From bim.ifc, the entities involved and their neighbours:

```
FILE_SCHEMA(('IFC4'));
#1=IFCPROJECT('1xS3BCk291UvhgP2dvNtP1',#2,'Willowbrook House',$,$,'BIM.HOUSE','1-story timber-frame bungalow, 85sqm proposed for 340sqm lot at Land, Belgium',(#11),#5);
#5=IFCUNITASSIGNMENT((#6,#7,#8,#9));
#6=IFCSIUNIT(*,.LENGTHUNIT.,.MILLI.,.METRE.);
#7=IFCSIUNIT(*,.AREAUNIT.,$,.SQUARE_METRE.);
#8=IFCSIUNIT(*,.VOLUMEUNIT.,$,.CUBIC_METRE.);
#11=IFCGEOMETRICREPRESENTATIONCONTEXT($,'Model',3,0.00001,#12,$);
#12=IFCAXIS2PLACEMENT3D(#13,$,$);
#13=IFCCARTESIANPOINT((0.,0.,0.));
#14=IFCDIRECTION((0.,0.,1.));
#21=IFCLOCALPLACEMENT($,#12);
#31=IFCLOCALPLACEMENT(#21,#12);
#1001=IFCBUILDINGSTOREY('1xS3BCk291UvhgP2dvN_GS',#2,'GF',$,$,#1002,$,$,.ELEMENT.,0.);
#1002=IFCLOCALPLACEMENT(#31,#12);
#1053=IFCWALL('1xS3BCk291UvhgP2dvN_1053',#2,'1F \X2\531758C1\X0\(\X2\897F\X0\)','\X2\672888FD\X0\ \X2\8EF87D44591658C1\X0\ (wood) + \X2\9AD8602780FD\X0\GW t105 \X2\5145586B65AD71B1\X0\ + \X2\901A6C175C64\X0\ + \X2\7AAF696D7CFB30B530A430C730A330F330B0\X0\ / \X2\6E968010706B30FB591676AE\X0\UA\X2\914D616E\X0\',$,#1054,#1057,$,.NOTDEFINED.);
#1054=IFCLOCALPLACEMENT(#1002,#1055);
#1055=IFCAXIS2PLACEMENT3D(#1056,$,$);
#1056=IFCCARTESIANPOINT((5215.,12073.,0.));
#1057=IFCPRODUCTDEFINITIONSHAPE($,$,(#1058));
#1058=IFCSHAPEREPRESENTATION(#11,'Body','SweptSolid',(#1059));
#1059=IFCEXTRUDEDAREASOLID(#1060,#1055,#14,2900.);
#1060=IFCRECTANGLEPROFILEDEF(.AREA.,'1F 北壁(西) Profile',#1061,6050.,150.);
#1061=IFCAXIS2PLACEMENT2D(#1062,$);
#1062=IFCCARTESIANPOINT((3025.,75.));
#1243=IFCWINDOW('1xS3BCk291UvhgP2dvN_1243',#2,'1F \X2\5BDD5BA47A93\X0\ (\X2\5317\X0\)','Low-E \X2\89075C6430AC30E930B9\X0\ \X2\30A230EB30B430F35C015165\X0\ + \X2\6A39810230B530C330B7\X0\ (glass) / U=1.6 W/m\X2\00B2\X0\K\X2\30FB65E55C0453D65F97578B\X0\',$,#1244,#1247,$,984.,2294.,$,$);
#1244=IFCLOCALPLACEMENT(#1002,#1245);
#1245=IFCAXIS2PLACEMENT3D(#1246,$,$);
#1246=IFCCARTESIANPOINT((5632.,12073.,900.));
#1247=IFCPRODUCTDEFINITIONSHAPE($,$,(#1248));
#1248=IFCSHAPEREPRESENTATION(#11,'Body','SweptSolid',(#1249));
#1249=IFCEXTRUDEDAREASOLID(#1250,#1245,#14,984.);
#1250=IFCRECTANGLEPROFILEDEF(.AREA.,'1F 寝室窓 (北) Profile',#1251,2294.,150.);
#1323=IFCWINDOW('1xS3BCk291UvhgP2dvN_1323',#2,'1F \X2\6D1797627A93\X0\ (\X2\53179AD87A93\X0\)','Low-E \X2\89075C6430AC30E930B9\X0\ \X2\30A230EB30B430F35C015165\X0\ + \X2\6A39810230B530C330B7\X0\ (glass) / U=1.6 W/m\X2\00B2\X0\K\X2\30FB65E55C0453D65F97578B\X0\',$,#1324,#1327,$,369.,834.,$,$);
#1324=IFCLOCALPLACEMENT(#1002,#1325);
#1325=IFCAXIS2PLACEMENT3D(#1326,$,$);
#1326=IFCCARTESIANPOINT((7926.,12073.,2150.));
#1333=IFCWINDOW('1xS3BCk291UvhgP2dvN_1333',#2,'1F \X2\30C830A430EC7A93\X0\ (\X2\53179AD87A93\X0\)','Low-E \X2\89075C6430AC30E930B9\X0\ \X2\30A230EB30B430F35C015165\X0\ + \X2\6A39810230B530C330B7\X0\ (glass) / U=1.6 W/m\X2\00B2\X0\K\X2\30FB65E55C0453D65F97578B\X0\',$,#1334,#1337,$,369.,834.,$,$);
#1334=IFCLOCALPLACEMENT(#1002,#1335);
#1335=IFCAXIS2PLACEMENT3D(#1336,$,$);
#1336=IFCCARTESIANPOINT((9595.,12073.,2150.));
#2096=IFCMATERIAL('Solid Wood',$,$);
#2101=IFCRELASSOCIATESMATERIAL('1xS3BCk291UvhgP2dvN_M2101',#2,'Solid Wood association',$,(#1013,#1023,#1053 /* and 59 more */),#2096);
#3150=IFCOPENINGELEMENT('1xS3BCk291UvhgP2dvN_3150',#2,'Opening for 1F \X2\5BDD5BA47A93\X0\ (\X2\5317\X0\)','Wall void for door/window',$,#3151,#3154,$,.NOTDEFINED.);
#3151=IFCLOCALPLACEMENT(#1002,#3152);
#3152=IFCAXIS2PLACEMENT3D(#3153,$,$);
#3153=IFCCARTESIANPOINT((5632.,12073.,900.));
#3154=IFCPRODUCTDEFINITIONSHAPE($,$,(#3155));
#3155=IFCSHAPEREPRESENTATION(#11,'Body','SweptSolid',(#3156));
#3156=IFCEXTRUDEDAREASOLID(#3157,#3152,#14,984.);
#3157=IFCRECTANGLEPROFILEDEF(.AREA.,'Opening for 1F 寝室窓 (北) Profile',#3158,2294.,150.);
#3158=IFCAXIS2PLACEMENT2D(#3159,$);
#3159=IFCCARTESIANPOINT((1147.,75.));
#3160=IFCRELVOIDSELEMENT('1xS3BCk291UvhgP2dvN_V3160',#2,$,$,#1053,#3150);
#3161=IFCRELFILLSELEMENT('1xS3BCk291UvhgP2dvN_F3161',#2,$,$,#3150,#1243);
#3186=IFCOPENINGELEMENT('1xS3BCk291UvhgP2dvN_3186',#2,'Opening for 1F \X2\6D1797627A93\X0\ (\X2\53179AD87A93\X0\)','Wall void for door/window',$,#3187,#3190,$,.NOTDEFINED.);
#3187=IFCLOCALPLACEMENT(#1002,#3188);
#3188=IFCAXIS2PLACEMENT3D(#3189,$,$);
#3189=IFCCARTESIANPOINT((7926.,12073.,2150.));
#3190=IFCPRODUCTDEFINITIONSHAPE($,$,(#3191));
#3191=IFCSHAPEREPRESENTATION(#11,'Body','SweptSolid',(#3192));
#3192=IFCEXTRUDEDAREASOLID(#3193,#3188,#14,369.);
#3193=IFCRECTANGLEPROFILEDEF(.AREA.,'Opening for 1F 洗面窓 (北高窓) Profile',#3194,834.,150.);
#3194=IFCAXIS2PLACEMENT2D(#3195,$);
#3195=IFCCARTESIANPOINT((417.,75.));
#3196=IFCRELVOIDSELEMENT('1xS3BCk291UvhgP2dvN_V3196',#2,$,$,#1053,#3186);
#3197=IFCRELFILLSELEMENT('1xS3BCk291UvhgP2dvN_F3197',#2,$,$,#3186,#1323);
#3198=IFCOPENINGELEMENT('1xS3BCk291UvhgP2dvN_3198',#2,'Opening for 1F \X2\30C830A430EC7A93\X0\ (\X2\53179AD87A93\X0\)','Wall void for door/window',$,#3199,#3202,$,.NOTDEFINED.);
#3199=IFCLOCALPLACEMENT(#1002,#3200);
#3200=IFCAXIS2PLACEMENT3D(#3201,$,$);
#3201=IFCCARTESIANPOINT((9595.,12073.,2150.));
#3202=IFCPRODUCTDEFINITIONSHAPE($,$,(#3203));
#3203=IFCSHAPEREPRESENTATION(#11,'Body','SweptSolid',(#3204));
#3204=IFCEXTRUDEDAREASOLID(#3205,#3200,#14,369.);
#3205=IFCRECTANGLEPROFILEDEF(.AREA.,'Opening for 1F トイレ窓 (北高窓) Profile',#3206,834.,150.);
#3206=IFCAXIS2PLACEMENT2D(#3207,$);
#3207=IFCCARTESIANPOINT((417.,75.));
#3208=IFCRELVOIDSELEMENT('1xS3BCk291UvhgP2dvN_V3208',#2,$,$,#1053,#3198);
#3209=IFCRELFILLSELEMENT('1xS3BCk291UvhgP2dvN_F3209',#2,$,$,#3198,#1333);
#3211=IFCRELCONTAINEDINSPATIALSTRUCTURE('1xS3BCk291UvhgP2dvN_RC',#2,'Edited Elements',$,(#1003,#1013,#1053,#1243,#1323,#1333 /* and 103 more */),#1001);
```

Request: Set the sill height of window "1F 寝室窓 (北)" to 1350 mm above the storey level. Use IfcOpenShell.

```python
import numpy as np
import ifcopenshell
import ifcopenshell.api.geometry
import ifcopenshell.geom
import ifcopenshell.util.element
import ifcopenshell.util.placement
import ifcopenshell.util.shape
import ifcopenshell.util.unit

model = ifcopenshell.open("bim.ifc")
unit_scale = ifcopenshell.util.unit.calculate_unit_scale(model)

window = model.by_guid("1xS3BCk291UvhgP2dvN_1243")
opening = window.FillsVoids[0].RelatingOpeningElement
storey = ifcopenshell.util.element.get_container(window, ifc_class="IfcBuildingStorey")
level = ifcopenshell.util.placement.get_local_placement(storey.ObjectPlacement)[2, 3]

# The opening's origin need not be at the sill, so measure its lowest point.
shape = ifcopenshell.geom.create_shape(ifcopenshell.geom.settings(), opening)
bottom = ifcopenshell.util.shape.get_shape_bottom_elevation(shape, shape.geometry) / unit_scale
dz = level + 1.35 / unit_scale - bottom

shift = np.array([0.0, 0.0, dz])
# The window is not placed relative to its opening, so move both.
for product in (opening, window):
    matrix = ifcopenshell.util.placement.get_local_placement(product.ObjectPlacement)
    matrix[:3, 3] += shift
    ifcopenshell.api.geometry.edit_object_placement(model, product=product, matrix=matrix, is_si=False)

print(f"moved by {dz * unit_scale:+.3f} m")

model.write("bim_rev.ifc")
```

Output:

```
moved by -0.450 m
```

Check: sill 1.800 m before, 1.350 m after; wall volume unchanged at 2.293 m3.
